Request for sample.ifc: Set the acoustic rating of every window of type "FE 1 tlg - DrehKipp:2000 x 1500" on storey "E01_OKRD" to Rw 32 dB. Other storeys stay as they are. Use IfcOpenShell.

First a look at what the model holds.

```python
import ifcopenshell
import ifcopenshell.util.element

model = ifcopenshell.open("sample.ifc")
print(model.schema)
storey = next(s for s in model.by_type("IfcBuildingStorey") if s.Name == "E01_OKRD")
windows = [e for e in ifcopenshell.util.element.get_decomposition(storey) if e.is_a("IfcWindow")]
seen = {}
for e in windows:
    element_type = ifcopenshell.util.element.get_type(e)
    key = (element_type.Name if element_type != e and element_type else None, ifcopenshell.util.element.get_pset(e, "Pset_WindowCommon", "AcousticRating"))
    seen[key] = seen.get(key, 0) + 1
for (name, value), count in sorted(seen.items(), key=str):
    print(count, "x", name, "|", value)
```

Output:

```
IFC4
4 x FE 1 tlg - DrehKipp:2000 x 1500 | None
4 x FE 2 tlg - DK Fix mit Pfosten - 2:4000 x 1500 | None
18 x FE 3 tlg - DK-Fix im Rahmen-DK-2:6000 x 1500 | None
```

```python
import ifcopenshell
import ifcopenshell.api.pset
import ifcopenshell.util.element

model = ifcopenshell.open("sample.ifc")

storey = next(s for s in model.by_type("IfcBuildingStorey") if s.Name == "E01_OKRD")
windows = [e for e in ifcopenshell.util.element.get_decomposition(storey) if e.is_a("IfcWindow")]

count = 0
for e in windows:
    element_type = ifcopenshell.util.element.get_type(e)
    if element_type in (None, e) or element_type.Name != "FE 1 tlg - DrehKipp:2000 x 1500":
        continue
    # add_pset returns the element's existing set when there is one.
    pset = ifcopenshell.api.pset.add_pset(model, product=e, name="Pset_WindowCommon")
    ifcopenshell.api.pset.edit_pset(model, pset=pset, properties={"AcousticRating": "Rw 32 dB"})
    count += 1

print(count, "windows updated")

model.write("sample_edited.ifc")
```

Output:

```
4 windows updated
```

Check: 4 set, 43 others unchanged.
